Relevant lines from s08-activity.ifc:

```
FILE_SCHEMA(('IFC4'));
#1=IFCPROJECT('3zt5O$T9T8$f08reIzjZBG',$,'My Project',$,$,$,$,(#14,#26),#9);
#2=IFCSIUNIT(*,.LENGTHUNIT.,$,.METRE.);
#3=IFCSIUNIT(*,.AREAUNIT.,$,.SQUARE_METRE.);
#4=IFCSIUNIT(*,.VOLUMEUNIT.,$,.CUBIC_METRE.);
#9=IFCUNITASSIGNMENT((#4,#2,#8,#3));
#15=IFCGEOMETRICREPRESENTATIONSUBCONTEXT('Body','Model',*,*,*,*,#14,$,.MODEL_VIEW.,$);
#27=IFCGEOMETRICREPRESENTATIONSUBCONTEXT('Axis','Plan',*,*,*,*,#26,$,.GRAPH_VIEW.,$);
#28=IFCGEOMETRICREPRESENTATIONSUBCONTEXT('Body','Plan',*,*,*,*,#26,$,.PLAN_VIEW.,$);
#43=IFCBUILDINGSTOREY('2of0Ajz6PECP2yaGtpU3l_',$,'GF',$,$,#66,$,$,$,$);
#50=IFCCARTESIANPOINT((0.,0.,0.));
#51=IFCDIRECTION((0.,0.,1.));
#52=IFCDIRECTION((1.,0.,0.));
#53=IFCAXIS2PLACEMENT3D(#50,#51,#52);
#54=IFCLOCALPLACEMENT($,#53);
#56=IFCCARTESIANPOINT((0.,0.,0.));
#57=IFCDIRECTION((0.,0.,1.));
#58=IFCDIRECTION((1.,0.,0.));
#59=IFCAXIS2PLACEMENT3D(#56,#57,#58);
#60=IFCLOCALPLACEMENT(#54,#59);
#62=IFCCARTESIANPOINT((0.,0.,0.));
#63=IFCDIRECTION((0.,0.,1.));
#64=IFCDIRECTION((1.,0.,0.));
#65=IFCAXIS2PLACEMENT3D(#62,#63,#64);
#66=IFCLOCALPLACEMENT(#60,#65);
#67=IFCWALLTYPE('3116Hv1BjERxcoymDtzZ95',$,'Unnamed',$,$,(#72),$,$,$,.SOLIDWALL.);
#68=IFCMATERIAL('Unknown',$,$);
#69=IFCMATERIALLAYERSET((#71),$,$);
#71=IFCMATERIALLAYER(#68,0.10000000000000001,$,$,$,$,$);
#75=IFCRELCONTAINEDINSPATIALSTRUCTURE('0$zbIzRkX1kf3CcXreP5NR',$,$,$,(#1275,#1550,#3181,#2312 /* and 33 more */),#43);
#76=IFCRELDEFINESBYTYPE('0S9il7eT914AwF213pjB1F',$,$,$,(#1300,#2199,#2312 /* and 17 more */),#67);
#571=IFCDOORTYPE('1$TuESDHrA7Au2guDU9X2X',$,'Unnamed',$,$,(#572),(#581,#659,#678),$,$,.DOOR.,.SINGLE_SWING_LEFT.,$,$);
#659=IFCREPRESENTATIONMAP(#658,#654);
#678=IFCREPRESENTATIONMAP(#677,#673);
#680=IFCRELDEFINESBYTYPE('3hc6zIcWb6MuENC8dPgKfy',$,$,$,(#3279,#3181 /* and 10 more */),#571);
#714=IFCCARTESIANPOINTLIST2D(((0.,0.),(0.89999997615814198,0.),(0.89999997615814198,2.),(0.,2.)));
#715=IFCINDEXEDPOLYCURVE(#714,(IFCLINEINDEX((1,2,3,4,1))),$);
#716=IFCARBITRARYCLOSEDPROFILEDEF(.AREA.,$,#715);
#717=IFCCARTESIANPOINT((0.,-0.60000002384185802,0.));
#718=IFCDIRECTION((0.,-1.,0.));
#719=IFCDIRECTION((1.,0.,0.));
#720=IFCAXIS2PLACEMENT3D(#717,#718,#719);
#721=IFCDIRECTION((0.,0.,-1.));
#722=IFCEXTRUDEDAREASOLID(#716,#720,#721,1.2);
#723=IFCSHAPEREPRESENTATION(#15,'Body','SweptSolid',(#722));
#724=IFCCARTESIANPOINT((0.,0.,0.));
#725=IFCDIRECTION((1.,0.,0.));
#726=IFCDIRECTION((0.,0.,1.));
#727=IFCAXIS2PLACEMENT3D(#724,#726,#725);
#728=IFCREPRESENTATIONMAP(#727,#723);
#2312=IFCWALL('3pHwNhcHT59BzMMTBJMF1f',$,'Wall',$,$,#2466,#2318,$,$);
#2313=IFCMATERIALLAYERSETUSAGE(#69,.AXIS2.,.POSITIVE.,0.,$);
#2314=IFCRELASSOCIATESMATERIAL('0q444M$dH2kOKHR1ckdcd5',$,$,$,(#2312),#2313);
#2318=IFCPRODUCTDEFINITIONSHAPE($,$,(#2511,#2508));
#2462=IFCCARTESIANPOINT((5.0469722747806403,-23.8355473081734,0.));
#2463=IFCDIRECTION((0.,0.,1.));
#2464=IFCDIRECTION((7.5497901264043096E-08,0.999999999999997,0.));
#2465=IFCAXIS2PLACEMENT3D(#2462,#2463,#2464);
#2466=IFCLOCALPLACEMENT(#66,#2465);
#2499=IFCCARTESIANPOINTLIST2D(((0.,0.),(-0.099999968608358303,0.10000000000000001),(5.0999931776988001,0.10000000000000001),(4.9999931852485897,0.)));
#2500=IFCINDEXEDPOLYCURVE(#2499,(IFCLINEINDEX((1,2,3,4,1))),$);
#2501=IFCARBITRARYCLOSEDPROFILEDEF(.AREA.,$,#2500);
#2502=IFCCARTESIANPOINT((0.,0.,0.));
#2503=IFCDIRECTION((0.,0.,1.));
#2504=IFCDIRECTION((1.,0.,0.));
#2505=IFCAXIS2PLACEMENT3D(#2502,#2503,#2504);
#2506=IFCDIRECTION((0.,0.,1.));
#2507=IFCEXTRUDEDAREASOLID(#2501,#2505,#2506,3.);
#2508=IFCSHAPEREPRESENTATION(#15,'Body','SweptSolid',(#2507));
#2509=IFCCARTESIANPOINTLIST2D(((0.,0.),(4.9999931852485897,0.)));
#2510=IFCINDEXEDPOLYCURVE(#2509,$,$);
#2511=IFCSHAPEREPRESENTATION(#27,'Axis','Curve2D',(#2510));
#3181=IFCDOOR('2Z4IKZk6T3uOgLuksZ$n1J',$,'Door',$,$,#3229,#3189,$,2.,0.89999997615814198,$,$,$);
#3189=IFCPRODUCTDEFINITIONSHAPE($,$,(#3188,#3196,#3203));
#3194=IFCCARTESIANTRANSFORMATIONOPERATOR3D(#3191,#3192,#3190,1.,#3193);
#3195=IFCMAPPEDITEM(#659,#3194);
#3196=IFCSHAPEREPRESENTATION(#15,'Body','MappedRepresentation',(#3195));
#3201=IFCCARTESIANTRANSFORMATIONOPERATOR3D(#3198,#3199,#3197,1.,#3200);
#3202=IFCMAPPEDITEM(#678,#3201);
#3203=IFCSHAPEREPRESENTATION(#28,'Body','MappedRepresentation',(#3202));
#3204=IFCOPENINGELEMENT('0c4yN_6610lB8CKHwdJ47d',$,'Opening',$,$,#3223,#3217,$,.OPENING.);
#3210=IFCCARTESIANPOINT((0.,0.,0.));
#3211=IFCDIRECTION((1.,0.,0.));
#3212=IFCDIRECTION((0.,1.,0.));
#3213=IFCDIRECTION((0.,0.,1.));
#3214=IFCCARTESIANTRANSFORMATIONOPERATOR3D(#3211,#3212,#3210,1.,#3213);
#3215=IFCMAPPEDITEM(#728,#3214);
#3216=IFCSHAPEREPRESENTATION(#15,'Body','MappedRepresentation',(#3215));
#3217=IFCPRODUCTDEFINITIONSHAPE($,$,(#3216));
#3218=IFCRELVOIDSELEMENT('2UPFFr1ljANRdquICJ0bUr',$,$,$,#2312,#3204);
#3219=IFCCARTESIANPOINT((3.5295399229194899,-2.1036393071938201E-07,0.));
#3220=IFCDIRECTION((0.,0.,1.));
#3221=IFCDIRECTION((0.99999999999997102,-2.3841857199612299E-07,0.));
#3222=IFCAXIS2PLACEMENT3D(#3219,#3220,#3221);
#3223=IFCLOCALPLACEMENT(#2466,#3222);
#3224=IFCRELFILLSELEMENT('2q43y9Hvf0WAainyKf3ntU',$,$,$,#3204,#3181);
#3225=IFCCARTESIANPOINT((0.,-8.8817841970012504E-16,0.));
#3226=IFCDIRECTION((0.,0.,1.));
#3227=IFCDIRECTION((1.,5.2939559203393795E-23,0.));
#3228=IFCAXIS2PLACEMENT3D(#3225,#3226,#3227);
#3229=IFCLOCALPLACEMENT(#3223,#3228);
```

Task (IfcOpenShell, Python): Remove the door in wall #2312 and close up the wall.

```python
import ifcopenshell
import ifcopenshell.api.feature
import ifcopenshell.api.root
import ifcopenshell.geom
import ifcopenshell.util.shape

model = ifcopenshell.open("s08-activity.ifc")
settings = ifcopenshell.geom.settings()


def volume(element):
    """Net volume in cubic metres, openings subtracted."""
    shape = ifcopenshell.geom.create_shape(settings, element)
    return ifcopenshell.util.shape.get_volume(shape.geometry)


door = model.by_id(3181)
opening = door.FillsVoids[0].RelatingOpeningElement
wall = opening.VoidsElements[0].RelatingBuildingElement
before = volume(wall)

ifcopenshell.api.root.remove_product(model, product=door)
ifcopenshell.api.feature.remove_feature(model, feature=opening)

after = volume(wall)

print(f"wall volume {before:.3f} -> {after:.3f} m3")

model.write("s08-activity-out.ifc")
```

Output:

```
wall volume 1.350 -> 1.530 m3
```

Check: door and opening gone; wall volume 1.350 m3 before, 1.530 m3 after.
